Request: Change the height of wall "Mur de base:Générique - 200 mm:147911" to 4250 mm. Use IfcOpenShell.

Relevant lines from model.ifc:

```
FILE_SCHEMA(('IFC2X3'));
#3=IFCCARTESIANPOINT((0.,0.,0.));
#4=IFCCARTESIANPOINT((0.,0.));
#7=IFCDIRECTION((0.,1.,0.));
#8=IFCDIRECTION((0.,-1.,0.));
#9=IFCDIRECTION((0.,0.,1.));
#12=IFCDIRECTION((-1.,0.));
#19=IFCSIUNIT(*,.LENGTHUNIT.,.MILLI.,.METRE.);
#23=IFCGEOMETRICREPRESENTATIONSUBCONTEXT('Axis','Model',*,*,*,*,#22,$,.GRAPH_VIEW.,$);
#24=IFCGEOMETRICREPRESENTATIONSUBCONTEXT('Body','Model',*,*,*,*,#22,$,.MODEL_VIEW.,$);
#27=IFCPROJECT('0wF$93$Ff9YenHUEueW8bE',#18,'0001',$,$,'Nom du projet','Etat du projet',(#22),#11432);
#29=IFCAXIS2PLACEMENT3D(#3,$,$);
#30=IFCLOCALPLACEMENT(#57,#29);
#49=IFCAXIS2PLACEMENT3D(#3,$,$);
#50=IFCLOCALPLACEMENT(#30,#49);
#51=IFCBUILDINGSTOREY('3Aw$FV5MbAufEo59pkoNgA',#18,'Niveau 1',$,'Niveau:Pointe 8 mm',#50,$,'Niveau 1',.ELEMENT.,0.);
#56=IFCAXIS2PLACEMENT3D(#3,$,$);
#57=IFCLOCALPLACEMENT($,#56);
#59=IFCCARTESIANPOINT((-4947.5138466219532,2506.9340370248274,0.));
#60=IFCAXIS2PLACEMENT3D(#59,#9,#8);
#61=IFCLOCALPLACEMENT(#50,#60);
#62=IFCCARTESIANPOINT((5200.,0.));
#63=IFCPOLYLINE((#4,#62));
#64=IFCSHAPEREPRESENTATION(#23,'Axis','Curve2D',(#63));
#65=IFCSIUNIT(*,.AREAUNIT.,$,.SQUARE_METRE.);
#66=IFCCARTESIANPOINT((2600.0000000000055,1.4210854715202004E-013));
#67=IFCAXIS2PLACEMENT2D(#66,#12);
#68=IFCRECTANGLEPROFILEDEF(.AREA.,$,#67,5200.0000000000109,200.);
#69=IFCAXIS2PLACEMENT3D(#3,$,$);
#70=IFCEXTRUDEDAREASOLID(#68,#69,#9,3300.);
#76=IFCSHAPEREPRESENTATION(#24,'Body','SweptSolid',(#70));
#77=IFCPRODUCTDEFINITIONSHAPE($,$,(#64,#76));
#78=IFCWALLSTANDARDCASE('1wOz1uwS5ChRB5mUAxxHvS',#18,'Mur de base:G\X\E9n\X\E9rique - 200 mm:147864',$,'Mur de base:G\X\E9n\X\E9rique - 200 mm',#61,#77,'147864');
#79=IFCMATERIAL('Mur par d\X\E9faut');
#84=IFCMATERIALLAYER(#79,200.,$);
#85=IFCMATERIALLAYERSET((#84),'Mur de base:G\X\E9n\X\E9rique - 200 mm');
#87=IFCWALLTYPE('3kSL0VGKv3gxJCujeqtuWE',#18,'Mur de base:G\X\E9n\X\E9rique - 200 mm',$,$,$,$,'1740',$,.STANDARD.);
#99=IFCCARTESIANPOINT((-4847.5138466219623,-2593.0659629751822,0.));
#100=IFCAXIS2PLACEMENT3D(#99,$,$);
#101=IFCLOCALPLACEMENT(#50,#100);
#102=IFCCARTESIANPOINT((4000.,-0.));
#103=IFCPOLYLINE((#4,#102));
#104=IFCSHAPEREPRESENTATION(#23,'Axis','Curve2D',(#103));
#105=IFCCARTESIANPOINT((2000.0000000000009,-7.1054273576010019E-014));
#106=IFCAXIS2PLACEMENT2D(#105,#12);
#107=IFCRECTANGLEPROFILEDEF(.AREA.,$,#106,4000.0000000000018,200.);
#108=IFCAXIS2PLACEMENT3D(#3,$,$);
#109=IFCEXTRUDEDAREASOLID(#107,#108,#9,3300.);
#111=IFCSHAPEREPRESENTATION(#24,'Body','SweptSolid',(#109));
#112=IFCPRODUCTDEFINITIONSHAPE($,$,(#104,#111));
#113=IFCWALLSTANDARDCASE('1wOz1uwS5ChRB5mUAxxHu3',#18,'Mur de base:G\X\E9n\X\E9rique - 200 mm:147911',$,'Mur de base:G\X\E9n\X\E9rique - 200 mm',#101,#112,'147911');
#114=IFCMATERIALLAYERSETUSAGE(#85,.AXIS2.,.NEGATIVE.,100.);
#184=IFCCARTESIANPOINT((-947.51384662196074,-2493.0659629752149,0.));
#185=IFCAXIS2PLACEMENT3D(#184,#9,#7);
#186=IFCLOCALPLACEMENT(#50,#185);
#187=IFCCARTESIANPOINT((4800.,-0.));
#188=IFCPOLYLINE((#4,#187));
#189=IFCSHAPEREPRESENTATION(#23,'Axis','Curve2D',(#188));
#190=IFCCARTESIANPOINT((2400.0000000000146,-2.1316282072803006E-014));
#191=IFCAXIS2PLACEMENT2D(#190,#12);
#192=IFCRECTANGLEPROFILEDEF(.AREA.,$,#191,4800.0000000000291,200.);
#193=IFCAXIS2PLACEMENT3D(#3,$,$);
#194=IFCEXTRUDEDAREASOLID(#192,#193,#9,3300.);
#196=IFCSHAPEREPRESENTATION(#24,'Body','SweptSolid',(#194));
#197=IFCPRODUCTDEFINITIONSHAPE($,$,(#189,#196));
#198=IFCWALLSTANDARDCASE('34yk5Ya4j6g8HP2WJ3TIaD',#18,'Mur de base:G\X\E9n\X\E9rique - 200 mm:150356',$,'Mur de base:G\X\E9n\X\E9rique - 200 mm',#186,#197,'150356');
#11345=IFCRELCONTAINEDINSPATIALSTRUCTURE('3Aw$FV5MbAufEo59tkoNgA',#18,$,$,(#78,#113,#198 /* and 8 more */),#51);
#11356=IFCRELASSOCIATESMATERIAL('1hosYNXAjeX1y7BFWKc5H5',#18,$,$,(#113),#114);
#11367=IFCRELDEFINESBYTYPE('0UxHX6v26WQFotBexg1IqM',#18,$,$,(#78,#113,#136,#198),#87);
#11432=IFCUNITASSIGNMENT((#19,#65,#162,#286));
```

```python
import ifcopenshell
import ifcopenshell.geom
import ifcopenshell.util.representation
import ifcopenshell.util.shape
import ifcopenshell.util.unit

model = ifcopenshell.open("model.ifc")
unit_scale = ifcopenshell.util.unit.calculate_unit_scale(model)
settings = ifcopenshell.geom.settings()


def volume(element):
    """Net volume in cubic metres, openings subtracted."""
    shape = ifcopenshell.geom.create_shape(settings, element)
    return ifcopenshell.util.shape.get_volume(shape.geometry)


wall = model.by_guid("1wOz1uwS5ChRB5mUAxxHu3")
before = volume(wall)

body = ifcopenshell.util.representation.get_representation(wall, "Model", "Body")
solid = body.Items[0]
old_height = solid.Depth
solid.Depth = 4.25 / unit_scale
after = volume(wall)

print(f"height {old_height:g} -> {solid.Depth:g}, volume {before:.3f} -> {after:.3f} m3")

model.write("model-out.ifc")
```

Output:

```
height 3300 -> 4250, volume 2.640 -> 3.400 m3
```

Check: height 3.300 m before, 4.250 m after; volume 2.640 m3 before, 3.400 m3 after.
